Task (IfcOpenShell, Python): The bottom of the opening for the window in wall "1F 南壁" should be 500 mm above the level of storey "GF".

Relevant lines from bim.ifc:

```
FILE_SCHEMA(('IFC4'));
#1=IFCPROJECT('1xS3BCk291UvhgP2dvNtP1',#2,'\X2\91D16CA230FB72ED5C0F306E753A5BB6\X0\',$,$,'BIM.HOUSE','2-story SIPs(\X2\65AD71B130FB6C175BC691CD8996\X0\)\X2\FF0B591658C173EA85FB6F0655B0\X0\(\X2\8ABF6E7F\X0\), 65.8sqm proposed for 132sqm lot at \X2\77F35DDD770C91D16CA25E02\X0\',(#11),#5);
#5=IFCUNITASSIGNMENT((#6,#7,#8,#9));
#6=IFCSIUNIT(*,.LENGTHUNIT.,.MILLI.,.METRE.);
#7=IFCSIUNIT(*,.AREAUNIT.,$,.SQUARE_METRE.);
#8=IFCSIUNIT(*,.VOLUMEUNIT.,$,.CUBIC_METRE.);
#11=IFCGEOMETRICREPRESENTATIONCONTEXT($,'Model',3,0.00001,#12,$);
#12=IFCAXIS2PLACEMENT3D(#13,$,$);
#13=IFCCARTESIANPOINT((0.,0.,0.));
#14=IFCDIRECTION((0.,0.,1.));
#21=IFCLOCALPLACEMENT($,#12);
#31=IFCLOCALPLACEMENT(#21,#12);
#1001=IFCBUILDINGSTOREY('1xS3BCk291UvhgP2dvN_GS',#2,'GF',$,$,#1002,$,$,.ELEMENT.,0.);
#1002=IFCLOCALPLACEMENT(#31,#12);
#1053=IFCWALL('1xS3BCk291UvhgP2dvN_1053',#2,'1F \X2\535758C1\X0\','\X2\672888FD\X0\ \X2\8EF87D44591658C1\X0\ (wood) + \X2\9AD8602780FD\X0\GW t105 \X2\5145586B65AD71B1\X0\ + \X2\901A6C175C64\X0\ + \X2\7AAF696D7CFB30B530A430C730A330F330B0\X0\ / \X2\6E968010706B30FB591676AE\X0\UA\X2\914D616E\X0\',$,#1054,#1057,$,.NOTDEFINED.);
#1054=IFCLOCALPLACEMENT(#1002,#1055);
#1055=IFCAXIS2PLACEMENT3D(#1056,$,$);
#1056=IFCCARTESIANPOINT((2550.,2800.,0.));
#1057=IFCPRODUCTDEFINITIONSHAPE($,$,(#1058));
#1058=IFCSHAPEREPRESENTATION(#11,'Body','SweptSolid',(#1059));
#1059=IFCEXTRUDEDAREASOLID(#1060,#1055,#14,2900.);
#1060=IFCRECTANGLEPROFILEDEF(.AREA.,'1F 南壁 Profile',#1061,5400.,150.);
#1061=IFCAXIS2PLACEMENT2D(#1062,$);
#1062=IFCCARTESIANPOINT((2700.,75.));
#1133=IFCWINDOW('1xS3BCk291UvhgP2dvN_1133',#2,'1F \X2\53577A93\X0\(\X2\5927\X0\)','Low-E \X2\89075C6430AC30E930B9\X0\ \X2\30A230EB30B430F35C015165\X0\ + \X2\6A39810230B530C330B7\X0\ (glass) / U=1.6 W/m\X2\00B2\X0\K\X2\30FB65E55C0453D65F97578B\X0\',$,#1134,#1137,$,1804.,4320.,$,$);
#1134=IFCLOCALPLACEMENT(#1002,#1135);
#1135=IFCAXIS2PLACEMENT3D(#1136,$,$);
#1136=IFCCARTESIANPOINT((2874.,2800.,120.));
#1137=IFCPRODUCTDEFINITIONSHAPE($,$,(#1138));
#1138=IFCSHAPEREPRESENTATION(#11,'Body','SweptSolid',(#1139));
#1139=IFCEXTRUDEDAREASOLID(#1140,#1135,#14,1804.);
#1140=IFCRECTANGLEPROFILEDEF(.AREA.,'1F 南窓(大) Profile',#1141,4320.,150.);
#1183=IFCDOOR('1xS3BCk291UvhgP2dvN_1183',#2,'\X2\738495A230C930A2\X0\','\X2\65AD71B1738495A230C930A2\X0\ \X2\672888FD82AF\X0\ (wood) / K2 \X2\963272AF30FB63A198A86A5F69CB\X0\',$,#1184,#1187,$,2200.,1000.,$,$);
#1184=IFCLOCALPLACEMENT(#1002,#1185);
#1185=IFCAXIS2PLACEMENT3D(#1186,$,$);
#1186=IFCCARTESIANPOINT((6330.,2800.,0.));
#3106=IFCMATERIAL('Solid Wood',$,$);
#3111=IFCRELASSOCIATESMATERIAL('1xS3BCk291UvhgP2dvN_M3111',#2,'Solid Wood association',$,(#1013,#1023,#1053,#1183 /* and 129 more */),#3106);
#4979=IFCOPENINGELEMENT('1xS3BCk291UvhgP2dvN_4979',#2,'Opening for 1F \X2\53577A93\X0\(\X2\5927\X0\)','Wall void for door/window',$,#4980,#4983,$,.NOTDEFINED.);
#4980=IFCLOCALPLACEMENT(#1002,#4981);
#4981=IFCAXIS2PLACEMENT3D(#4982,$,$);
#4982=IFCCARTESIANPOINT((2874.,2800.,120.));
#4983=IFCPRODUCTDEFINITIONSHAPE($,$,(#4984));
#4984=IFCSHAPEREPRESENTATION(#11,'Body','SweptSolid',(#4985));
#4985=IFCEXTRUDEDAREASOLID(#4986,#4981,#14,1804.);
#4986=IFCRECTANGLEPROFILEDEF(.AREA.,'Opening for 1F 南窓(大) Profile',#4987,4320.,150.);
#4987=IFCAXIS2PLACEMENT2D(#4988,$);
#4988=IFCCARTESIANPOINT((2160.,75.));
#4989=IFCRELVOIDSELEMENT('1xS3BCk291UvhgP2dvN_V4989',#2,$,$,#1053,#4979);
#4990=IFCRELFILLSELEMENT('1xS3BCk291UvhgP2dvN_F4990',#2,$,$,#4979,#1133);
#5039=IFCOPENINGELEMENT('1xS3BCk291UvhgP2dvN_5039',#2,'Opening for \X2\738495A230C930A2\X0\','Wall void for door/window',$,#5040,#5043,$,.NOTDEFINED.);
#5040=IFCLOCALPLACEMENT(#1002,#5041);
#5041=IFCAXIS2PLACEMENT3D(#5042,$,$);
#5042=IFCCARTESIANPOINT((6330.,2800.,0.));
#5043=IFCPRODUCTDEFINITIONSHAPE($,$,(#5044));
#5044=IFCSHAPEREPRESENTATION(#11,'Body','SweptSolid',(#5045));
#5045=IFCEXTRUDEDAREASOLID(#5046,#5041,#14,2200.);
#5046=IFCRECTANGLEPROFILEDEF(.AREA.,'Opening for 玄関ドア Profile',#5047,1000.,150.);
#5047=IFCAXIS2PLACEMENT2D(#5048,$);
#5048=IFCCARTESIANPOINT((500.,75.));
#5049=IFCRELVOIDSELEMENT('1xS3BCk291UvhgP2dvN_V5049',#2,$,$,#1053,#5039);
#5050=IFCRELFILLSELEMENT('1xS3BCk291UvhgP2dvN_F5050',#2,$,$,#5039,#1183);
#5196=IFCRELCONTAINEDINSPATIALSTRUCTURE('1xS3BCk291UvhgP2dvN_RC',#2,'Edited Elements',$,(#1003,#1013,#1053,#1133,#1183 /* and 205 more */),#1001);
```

```python
import numpy as np
import ifcopenshell
import ifcopenshell.api.geometry
import ifcopenshell.geom
import ifcopenshell.util.element
import ifcopenshell.util.placement
import ifcopenshell.util.shape
import ifcopenshell.util.unit

model = ifcopenshell.open("bim.ifc")
unit_scale = ifcopenshell.util.unit.calculate_unit_scale(model)

window = model.by_guid("1xS3BCk291UvhgP2dvN_1133")
opening = window.FillsVoids[0].RelatingOpeningElement
storey = ifcopenshell.util.element.get_container(window, ifc_class="IfcBuildingStorey")
level = ifcopenshell.util.placement.get_local_placement(storey.ObjectPlacement)[2, 3]

# The opening's origin need not be at the sill, so measure its lowest point.
shape = ifcopenshell.geom.create_shape(ifcopenshell.geom.settings(), opening)
bottom = ifcopenshell.util.shape.get_shape_bottom_elevation(shape, shape.geometry) / unit_scale
dz = level + 500.0 - bottom

shift = np.array([0.0, 0.0, dz])
# The window is not placed relative to its opening, so move both.
for product in (opening, window):
    matrix = ifcopenshell.util.placement.get_local_placement(product.ObjectPlacement)
    matrix[:3, 3] += shift
    ifcopenshell.api.geometry.edit_object_placement(model, product=product, matrix=matrix, is_si=False)

print(f"moved by {dz * unit_scale:+.3f} m")

model.write("bim_v2.ifc")
```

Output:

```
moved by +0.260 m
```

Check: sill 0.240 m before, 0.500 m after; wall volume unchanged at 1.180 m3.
